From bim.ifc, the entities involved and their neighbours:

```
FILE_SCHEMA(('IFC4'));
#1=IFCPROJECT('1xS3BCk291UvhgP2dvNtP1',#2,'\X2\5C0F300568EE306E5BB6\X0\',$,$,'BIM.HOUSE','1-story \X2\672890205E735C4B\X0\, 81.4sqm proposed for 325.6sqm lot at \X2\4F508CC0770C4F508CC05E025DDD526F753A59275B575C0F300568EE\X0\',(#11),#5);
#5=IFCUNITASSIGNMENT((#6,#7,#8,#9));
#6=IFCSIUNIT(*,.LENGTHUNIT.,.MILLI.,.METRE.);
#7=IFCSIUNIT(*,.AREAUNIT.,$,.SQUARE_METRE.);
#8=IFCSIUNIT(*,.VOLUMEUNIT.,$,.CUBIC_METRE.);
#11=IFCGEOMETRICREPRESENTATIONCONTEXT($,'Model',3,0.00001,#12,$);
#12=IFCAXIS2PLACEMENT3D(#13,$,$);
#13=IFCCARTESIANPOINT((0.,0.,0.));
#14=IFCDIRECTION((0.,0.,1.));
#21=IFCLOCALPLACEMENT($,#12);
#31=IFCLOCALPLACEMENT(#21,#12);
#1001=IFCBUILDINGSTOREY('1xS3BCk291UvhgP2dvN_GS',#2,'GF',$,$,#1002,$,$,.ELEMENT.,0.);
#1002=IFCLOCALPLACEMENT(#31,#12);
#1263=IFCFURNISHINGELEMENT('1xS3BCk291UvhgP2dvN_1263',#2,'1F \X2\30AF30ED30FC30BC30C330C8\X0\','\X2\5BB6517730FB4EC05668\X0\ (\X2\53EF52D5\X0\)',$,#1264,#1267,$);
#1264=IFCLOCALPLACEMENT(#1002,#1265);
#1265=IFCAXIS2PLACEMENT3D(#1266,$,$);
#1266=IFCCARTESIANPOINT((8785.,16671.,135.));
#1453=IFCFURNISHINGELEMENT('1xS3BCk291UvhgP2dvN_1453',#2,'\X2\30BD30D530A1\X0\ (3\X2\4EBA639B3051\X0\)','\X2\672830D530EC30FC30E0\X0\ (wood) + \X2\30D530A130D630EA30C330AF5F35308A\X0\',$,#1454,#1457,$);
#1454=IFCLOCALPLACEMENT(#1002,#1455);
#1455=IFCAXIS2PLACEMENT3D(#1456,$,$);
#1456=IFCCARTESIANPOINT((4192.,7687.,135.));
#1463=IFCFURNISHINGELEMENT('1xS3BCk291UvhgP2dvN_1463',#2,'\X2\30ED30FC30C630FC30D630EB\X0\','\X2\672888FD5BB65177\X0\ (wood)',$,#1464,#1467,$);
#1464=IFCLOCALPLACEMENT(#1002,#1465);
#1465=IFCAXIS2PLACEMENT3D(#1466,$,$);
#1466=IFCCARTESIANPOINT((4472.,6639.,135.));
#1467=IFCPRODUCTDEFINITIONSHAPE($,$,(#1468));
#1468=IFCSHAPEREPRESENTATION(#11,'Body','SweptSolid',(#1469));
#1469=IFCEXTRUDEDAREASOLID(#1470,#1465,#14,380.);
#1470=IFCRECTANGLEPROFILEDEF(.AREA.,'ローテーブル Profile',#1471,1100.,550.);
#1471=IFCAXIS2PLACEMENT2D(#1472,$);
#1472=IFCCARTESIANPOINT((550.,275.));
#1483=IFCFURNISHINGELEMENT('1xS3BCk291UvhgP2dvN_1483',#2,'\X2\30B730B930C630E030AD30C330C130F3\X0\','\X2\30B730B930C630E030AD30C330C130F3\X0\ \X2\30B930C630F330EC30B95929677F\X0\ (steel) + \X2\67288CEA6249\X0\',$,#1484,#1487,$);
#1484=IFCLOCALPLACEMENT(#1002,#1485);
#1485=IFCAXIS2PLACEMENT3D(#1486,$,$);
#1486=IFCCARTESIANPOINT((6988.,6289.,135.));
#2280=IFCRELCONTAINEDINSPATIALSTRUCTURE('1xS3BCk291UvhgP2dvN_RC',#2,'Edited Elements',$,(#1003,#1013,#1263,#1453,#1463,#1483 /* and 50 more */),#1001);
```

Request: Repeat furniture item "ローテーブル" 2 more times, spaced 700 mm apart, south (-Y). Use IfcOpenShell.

```python
import numpy as np
import ifcopenshell
import ifcopenshell.api.geometry
import ifcopenshell.api.root
import ifcopenshell.util.element
import ifcopenshell.util.placement
import ifcopenshell.util.unit

model = ifcopenshell.open("bim.ifc")
unit_scale = ifcopenshell.util.unit.calculate_unit_scale(model)


def reuse_history(source, copy):
    """copy_class also copies each property set's owner history, people and application; keep the originals."""
    for rel in copy.IsDefinedBy:
        if rel.is_a("IfcRelDefinesByProperties") and (history := rel.RelatingPropertyDefinition.OwnerHistory):
            rel.RelatingPropertyDefinition.OwnerHistory = source.OwnerHistory
            ifcopenshell.util.element.remove_deep2(model, history)


source = model.by_guid("1xS3BCk291UvhgP2dvN_1463")
base = ifcopenshell.util.placement.get_local_placement(source.ObjectPlacement)
step = np.array([0.0, -1.0, 0.0]) * 0.7 / unit_scale

for i in range(1, 3):
    copy = ifcopenshell.api.root.copy_class(model, product=source)
    copy.Representation = ifcopenshell.util.element.copy_deep(
        model, source.Representation, exclude=["IfcGeometricRepresentationContext", "IfcRepresentationMap"]
    )
    reuse_history(source, copy)
    matrix = base.copy()
    matrix[:3, 3] += i * step
    print("added at", matrix[:3, 3].round(3) + 0.0)
    ifcopenshell.api.geometry.edit_object_placement(model, product=copy, matrix=matrix, is_si=False)

model.write("bim-out.ifc")
```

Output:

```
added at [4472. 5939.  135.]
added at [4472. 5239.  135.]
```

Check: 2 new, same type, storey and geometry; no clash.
